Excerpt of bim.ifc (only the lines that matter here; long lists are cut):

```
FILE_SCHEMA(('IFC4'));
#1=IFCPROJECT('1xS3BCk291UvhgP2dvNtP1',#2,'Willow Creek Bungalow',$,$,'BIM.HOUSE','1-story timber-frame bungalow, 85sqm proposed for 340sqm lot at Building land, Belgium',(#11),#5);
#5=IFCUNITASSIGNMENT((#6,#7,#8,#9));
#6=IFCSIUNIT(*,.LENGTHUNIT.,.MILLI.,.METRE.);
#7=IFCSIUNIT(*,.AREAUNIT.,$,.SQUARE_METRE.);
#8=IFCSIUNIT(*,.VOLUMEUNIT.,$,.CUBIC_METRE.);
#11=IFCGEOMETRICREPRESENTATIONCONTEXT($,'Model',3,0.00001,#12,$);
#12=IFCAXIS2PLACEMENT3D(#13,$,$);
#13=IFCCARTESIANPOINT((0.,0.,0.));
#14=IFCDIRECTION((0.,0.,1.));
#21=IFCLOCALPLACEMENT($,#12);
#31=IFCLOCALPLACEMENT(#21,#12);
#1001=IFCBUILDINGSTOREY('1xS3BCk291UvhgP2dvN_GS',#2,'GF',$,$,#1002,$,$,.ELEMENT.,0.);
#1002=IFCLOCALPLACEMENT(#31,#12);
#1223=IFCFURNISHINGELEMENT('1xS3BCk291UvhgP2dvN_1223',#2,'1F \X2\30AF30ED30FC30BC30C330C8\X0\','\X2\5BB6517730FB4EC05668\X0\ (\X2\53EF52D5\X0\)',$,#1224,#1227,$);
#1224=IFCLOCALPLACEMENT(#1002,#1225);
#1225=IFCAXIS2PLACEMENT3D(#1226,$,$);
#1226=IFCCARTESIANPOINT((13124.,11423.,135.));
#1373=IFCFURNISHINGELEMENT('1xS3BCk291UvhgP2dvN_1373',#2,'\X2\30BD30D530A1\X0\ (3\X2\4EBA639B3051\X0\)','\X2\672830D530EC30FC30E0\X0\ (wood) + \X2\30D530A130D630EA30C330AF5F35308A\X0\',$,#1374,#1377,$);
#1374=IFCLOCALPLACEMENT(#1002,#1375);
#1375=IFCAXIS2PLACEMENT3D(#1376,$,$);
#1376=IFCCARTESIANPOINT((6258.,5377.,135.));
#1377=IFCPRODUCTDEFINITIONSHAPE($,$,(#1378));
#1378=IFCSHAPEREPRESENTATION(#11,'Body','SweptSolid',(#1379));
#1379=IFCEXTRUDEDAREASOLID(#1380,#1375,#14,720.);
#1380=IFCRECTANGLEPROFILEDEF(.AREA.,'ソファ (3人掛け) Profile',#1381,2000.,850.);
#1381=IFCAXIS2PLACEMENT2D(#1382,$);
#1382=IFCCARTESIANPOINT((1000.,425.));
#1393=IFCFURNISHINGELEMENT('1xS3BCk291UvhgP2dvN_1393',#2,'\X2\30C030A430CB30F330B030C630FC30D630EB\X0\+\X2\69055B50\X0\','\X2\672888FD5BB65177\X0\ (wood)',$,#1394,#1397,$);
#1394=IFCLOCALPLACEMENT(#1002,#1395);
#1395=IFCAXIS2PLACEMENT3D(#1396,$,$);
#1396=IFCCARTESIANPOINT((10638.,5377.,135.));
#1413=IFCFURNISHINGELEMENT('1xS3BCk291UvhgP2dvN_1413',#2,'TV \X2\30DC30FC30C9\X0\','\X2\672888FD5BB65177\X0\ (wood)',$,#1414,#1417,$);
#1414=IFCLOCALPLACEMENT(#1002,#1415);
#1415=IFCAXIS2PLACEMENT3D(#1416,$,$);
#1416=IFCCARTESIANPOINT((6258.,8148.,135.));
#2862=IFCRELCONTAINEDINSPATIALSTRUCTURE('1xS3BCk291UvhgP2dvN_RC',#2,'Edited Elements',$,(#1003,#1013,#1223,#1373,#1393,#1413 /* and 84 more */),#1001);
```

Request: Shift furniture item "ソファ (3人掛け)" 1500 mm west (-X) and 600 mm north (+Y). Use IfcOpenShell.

```python
import ifcopenshell
import ifcopenshell.api.geometry
import ifcopenshell.util.placement
import ifcopenshell.util.unit

model = ifcopenshell.open("bim.ifc")
unit_scale = ifcopenshell.util.unit.calculate_unit_scale(model)

item = model.by_id(1373)
matrix = ifcopenshell.util.placement.get_local_placement(item.ObjectPlacement)
matrix[0, 3] -= 1.5 / unit_scale
matrix[1, 3] += 0.6 / unit_scale
ifcopenshell.api.geometry.edit_object_placement(model, product=item, matrix=matrix, is_si=False)

print(ifcopenshell.util.placement.get_local_placement(item.ObjectPlacement).round(3) + 0.0)

model.write("bim_rev.ifc")
```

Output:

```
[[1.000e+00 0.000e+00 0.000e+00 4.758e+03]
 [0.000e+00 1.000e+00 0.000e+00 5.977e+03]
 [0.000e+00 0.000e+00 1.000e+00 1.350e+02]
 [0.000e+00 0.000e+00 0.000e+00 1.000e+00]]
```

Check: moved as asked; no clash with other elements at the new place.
